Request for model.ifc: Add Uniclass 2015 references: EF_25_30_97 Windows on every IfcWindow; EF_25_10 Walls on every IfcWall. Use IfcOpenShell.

First a look at what the model holds.

```python
import ifcopenshell

model = ifcopenshell.open("model.ifc")
print(model.schema)
print("classifications:", [c.Name for c in model.by_type("IfcClassification")])
for ifc_class in ("IfcDoor", "IfcRoof", "IfcStair", "IfcWall", "IfcWindow"):
    print(ifc_class, len(model.by_type(ifc_class)))
```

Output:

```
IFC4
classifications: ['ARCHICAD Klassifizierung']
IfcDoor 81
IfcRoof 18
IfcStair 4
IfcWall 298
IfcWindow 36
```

```python
import ifcopenshell
import ifcopenshell.api.classification

model = ifcopenshell.open("model.ifc")

system = ifcopenshell.api.classification.add_classification(model, classification="Uniclass 2015")

codes = {
    "IfcWindow": ("EF_25_30_97", "Windows"),
    "IfcWall": ("EF_25_10", "Walls"),
}
for ifc_class, (code, name) in codes.items():
    products = model.by_type(ifc_class)
    ifcopenshell.api.classification.add_reference(
        model, products=products, classification=system, identification=code, name=name
    )
    print(code, len(products))

model.write("model_updated.ifc")
```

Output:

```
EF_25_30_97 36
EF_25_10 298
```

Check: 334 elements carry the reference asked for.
